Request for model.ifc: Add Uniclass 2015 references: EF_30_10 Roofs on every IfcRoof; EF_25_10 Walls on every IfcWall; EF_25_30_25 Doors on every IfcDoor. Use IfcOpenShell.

First a look at what the model holds.

```python
import ifcopenshell

model = ifcopenshell.open("model.ifc")
print(model.schema)
print("classifications:", [c.Name for c in model.by_type("IfcClassification")])
for ifc_class in ("IfcDoor", "IfcRoof", "IfcStair", "IfcWall", "IfcWindow"):
    print(ifc_class, len(model.by_type(ifc_class)))
```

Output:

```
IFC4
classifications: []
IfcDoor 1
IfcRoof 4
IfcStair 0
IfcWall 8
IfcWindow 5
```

```python
import ifcopenshell
import ifcopenshell.api.classification

model = ifcopenshell.open("model.ifc")

system = ifcopenshell.api.classification.add_classification(model, classification="Uniclass 2015")

codes = {
    "IfcRoof": ("EF_30_10", "Roofs"),
    "IfcWall": ("EF_25_10", "Walls"),
    "IfcDoor": ("EF_25_30_25", "Doors"),
}
for ifc_class, (code, name) in codes.items():
    products = model.by_type(ifc_class)
    ifcopenshell.api.classification.add_reference(
        model, products=products, classification=system, identification=code, name=name
    )
    print(code, len(products))

model.write("model_rev.ifc")
```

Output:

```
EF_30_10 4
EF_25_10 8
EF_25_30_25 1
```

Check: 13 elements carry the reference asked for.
